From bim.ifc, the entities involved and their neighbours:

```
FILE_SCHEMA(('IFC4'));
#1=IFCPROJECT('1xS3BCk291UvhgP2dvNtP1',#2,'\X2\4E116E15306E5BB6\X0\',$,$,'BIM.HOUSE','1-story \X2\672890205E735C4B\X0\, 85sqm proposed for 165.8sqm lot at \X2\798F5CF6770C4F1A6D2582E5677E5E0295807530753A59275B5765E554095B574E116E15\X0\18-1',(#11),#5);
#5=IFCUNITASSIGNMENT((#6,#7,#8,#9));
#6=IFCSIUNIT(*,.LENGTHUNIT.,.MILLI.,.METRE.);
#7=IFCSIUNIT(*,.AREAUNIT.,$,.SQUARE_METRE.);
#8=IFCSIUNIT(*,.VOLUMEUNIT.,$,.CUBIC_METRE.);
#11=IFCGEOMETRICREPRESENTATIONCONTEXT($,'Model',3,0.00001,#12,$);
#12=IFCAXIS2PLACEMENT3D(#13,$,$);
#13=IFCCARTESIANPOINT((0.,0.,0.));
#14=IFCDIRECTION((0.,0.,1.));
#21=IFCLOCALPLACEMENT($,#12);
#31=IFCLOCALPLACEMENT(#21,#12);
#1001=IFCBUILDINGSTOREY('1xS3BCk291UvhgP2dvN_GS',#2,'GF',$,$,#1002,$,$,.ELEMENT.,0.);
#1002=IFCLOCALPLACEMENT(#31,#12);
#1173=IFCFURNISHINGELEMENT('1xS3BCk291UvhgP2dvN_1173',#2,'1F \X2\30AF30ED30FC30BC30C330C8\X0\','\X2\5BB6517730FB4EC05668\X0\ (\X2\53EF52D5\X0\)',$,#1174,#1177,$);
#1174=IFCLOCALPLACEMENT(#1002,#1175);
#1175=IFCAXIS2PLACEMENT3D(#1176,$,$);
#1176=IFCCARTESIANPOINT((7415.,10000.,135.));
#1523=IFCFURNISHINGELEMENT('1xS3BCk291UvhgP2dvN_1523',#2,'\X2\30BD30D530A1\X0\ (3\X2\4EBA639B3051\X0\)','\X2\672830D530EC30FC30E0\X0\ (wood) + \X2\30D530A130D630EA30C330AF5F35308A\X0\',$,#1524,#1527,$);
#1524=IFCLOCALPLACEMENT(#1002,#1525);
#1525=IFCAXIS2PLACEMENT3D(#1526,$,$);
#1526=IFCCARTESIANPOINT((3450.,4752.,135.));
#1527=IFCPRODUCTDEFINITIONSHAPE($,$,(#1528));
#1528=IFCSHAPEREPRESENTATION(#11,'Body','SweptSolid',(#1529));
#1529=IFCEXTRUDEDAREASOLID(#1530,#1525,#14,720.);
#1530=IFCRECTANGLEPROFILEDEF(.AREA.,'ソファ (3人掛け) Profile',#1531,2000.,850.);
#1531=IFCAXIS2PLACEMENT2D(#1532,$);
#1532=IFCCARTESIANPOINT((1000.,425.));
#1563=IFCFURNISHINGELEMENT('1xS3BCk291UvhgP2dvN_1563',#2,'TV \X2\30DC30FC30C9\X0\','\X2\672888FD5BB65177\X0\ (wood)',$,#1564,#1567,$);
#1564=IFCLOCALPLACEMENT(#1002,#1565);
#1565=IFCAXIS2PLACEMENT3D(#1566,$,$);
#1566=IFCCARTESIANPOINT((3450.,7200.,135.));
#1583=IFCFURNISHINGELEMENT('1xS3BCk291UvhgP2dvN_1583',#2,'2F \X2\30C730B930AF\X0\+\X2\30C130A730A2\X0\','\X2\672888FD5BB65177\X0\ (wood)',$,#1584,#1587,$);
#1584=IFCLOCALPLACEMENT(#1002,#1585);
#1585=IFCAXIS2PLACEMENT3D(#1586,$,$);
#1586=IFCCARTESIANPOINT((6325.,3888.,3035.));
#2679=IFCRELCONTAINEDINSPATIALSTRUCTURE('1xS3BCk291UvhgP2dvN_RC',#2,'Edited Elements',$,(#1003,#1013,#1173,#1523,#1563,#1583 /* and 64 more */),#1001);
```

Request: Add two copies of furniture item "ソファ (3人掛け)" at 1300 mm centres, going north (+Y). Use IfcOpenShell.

```python
import numpy as np
import ifcopenshell
import ifcopenshell.api.geometry
import ifcopenshell.api.root
import ifcopenshell.util.element
import ifcopenshell.util.placement

model = ifcopenshell.open("bim.ifc")


def reuse_history(source, copy):
    """copy_class also copies each property set's owner history, people and application; keep the originals."""
    for rel in copy.IsDefinedBy:
        if rel.is_a("IfcRelDefinesByProperties") and (history := rel.RelatingPropertyDefinition.OwnerHistory):
            rel.RelatingPropertyDefinition.OwnerHistory = source.OwnerHistory
            ifcopenshell.util.element.remove_deep2(model, history)


source = model.by_guid("1xS3BCk291UvhgP2dvN_1523")
base = ifcopenshell.util.placement.get_local_placement(source.ObjectPlacement)
step = np.array([0.0, 1.0, 0.0]) * 1300.0

for i in range(1, 3):
    copy = ifcopenshell.api.root.copy_class(model, product=source)
    copy.Representation = ifcopenshell.util.element.copy_deep(
        model, source.Representation, exclude=["IfcGeometricRepresentationContext", "IfcRepresentationMap"]
    )
    reuse_history(source, copy)
    matrix = base.copy()
    matrix[:3, 3] += i * step
    print("added at", matrix[:3, 3].round(3) + 0.0)
    ifcopenshell.api.geometry.edit_object_placement(model, product=copy, matrix=matrix, is_si=False)

model.write("bim_v2.ifc")
```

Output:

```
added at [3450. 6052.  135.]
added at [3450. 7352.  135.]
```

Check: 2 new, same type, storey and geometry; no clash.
